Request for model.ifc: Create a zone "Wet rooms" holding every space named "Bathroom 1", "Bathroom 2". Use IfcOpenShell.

First a look at what the model holds.

```python
import ifcopenshell

model = ifcopenshell.open("model.ifc")
print(model.schema)
seen = {}
for space in model.by_type("IfcSpace"):
    seen[space.LongName] = seen.get(space.LongName, 0) + 1
for name, count in sorted(seen.items(), key=str):
    print(count, "x", name)
print("zones:", [z.Name for z in model.by_type("IfcZone")][:20])
```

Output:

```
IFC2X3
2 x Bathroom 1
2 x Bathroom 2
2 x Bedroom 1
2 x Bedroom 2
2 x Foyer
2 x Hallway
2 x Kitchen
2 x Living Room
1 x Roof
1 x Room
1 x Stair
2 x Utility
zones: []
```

```python
import ifcopenshell
import ifcopenshell.api.group
import ifcopenshell.api.root

model = ifcopenshell.open("model.ifc")

names = {"Bathroom 1", "Bathroom 2"}
spaces = [s for s in model.by_type("IfcSpace") if s.LongName in names]

zone = ifcopenshell.api.root.create_entity(model, ifc_class="IfcZone", name="Wet rooms")
ifcopenshell.api.group.assign_group(model, products=spaces, group=zone)
print(len(spaces), "spaces in", zone.Name)

model.write("model_v2.ifc")
```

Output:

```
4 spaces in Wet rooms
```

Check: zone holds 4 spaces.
